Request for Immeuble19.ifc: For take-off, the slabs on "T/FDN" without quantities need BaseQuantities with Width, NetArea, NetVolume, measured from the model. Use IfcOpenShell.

First a look at what the model holds.

```python
import ifcopenshell
import ifcopenshell.util.element
import ifcopenshell.util.unit

model = ifcopenshell.open("Immeuble19.ifc")
print(model.schema)
for unit_type in ("LENGTHUNIT", "AREAUNIT", "VOLUMEUNIT"):
    print(unit_type, ifcopenshell.util.unit.calculate_unit_scale(model, unit_type))
storey = next(s for s in model.by_type("IfcBuildingStorey") if s.Name == "T/FDN")
slabs = [e for e in ifcopenshell.util.element.get_decomposition(storey) if e.is_a("IfcSlab")]
for e in sorted(slabs, key=lambda e: e.id()):
    print(e.id(), e.is_a(), e.Name, list(ifcopenshell.util.element.get_psets(e, qtos_only=True)), sep=" | ")
```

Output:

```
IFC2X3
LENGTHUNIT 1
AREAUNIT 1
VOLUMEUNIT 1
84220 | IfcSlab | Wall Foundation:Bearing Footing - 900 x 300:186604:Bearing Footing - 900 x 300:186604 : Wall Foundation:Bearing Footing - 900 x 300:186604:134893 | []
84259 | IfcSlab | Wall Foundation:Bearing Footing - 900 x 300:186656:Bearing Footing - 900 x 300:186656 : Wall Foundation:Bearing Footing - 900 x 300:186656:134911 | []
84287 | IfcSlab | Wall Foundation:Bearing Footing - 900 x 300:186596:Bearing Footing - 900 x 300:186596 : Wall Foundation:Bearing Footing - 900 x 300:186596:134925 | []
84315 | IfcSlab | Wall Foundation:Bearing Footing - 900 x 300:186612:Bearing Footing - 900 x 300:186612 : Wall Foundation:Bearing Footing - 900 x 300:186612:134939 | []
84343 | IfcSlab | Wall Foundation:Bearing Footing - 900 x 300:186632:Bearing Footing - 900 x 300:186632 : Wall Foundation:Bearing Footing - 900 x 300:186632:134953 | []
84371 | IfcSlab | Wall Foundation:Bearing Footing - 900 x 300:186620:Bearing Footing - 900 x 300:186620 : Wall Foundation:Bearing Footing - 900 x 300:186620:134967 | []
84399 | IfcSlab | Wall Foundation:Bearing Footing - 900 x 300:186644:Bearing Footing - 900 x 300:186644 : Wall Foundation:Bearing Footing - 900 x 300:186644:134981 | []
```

```python
import ifcopenshell
import ifcopenshell.api.pset
import ifcopenshell.geom
import ifcopenshell.util.element
import ifcopenshell.util.shape
import ifcopenshell.util.unit

model = ifcopenshell.open("Immeuble19.ifc")
unit_scale = ifcopenshell.util.unit.calculate_unit_scale(model)
area_scale = ifcopenshell.util.unit.calculate_unit_scale(model, "AREAUNIT")
volume_scale = ifcopenshell.util.unit.calculate_unit_scale(model, "VOLUMEUNIT")
settings = ifcopenshell.geom.settings()

storey = next(s for s in model.by_type("IfcBuildingStorey") if s.Name == "T/FDN")
slabs = [e for e in ifcopenshell.util.element.get_decomposition(storey) if e.is_a("IfcSlab")]

for e in sorted(slabs, key=lambda e: e.id()):
    if ifcopenshell.util.element.get_psets(e, qtos_only=True, should_inherit=False):
        continue
    # Geometry comes back in metres, in the element's own axes.
    shape = ifcopenshell.geom.create_shape(settings, e)
    values = {
        "Width": ifcopenshell.util.shape.get_z(shape.geometry) / unit_scale,
        "NetArea": ifcopenshell.util.shape.get_footprint_area(shape.geometry) / area_scale,
        "NetVolume": ifcopenshell.util.shape.get_volume(shape.geometry) / volume_scale,
    }
    qto = ifcopenshell.api.pset.add_qto(model, product=e, name="BaseQuantities")
    ifcopenshell.api.pset.edit_qto(model, qto=qto, properties=values)
    print(e.id(), {k: round(v, 3) for k, v in values.items()})

model.write("Immeuble19_rev.ifc")
```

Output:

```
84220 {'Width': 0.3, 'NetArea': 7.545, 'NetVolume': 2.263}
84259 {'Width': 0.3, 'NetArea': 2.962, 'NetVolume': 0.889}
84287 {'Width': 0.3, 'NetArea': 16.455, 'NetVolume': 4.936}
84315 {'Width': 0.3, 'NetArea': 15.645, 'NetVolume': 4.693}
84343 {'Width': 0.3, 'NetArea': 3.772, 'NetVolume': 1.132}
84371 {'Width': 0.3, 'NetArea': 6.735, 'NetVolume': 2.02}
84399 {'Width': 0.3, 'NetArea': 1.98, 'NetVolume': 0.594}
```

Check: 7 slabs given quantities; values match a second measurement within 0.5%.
